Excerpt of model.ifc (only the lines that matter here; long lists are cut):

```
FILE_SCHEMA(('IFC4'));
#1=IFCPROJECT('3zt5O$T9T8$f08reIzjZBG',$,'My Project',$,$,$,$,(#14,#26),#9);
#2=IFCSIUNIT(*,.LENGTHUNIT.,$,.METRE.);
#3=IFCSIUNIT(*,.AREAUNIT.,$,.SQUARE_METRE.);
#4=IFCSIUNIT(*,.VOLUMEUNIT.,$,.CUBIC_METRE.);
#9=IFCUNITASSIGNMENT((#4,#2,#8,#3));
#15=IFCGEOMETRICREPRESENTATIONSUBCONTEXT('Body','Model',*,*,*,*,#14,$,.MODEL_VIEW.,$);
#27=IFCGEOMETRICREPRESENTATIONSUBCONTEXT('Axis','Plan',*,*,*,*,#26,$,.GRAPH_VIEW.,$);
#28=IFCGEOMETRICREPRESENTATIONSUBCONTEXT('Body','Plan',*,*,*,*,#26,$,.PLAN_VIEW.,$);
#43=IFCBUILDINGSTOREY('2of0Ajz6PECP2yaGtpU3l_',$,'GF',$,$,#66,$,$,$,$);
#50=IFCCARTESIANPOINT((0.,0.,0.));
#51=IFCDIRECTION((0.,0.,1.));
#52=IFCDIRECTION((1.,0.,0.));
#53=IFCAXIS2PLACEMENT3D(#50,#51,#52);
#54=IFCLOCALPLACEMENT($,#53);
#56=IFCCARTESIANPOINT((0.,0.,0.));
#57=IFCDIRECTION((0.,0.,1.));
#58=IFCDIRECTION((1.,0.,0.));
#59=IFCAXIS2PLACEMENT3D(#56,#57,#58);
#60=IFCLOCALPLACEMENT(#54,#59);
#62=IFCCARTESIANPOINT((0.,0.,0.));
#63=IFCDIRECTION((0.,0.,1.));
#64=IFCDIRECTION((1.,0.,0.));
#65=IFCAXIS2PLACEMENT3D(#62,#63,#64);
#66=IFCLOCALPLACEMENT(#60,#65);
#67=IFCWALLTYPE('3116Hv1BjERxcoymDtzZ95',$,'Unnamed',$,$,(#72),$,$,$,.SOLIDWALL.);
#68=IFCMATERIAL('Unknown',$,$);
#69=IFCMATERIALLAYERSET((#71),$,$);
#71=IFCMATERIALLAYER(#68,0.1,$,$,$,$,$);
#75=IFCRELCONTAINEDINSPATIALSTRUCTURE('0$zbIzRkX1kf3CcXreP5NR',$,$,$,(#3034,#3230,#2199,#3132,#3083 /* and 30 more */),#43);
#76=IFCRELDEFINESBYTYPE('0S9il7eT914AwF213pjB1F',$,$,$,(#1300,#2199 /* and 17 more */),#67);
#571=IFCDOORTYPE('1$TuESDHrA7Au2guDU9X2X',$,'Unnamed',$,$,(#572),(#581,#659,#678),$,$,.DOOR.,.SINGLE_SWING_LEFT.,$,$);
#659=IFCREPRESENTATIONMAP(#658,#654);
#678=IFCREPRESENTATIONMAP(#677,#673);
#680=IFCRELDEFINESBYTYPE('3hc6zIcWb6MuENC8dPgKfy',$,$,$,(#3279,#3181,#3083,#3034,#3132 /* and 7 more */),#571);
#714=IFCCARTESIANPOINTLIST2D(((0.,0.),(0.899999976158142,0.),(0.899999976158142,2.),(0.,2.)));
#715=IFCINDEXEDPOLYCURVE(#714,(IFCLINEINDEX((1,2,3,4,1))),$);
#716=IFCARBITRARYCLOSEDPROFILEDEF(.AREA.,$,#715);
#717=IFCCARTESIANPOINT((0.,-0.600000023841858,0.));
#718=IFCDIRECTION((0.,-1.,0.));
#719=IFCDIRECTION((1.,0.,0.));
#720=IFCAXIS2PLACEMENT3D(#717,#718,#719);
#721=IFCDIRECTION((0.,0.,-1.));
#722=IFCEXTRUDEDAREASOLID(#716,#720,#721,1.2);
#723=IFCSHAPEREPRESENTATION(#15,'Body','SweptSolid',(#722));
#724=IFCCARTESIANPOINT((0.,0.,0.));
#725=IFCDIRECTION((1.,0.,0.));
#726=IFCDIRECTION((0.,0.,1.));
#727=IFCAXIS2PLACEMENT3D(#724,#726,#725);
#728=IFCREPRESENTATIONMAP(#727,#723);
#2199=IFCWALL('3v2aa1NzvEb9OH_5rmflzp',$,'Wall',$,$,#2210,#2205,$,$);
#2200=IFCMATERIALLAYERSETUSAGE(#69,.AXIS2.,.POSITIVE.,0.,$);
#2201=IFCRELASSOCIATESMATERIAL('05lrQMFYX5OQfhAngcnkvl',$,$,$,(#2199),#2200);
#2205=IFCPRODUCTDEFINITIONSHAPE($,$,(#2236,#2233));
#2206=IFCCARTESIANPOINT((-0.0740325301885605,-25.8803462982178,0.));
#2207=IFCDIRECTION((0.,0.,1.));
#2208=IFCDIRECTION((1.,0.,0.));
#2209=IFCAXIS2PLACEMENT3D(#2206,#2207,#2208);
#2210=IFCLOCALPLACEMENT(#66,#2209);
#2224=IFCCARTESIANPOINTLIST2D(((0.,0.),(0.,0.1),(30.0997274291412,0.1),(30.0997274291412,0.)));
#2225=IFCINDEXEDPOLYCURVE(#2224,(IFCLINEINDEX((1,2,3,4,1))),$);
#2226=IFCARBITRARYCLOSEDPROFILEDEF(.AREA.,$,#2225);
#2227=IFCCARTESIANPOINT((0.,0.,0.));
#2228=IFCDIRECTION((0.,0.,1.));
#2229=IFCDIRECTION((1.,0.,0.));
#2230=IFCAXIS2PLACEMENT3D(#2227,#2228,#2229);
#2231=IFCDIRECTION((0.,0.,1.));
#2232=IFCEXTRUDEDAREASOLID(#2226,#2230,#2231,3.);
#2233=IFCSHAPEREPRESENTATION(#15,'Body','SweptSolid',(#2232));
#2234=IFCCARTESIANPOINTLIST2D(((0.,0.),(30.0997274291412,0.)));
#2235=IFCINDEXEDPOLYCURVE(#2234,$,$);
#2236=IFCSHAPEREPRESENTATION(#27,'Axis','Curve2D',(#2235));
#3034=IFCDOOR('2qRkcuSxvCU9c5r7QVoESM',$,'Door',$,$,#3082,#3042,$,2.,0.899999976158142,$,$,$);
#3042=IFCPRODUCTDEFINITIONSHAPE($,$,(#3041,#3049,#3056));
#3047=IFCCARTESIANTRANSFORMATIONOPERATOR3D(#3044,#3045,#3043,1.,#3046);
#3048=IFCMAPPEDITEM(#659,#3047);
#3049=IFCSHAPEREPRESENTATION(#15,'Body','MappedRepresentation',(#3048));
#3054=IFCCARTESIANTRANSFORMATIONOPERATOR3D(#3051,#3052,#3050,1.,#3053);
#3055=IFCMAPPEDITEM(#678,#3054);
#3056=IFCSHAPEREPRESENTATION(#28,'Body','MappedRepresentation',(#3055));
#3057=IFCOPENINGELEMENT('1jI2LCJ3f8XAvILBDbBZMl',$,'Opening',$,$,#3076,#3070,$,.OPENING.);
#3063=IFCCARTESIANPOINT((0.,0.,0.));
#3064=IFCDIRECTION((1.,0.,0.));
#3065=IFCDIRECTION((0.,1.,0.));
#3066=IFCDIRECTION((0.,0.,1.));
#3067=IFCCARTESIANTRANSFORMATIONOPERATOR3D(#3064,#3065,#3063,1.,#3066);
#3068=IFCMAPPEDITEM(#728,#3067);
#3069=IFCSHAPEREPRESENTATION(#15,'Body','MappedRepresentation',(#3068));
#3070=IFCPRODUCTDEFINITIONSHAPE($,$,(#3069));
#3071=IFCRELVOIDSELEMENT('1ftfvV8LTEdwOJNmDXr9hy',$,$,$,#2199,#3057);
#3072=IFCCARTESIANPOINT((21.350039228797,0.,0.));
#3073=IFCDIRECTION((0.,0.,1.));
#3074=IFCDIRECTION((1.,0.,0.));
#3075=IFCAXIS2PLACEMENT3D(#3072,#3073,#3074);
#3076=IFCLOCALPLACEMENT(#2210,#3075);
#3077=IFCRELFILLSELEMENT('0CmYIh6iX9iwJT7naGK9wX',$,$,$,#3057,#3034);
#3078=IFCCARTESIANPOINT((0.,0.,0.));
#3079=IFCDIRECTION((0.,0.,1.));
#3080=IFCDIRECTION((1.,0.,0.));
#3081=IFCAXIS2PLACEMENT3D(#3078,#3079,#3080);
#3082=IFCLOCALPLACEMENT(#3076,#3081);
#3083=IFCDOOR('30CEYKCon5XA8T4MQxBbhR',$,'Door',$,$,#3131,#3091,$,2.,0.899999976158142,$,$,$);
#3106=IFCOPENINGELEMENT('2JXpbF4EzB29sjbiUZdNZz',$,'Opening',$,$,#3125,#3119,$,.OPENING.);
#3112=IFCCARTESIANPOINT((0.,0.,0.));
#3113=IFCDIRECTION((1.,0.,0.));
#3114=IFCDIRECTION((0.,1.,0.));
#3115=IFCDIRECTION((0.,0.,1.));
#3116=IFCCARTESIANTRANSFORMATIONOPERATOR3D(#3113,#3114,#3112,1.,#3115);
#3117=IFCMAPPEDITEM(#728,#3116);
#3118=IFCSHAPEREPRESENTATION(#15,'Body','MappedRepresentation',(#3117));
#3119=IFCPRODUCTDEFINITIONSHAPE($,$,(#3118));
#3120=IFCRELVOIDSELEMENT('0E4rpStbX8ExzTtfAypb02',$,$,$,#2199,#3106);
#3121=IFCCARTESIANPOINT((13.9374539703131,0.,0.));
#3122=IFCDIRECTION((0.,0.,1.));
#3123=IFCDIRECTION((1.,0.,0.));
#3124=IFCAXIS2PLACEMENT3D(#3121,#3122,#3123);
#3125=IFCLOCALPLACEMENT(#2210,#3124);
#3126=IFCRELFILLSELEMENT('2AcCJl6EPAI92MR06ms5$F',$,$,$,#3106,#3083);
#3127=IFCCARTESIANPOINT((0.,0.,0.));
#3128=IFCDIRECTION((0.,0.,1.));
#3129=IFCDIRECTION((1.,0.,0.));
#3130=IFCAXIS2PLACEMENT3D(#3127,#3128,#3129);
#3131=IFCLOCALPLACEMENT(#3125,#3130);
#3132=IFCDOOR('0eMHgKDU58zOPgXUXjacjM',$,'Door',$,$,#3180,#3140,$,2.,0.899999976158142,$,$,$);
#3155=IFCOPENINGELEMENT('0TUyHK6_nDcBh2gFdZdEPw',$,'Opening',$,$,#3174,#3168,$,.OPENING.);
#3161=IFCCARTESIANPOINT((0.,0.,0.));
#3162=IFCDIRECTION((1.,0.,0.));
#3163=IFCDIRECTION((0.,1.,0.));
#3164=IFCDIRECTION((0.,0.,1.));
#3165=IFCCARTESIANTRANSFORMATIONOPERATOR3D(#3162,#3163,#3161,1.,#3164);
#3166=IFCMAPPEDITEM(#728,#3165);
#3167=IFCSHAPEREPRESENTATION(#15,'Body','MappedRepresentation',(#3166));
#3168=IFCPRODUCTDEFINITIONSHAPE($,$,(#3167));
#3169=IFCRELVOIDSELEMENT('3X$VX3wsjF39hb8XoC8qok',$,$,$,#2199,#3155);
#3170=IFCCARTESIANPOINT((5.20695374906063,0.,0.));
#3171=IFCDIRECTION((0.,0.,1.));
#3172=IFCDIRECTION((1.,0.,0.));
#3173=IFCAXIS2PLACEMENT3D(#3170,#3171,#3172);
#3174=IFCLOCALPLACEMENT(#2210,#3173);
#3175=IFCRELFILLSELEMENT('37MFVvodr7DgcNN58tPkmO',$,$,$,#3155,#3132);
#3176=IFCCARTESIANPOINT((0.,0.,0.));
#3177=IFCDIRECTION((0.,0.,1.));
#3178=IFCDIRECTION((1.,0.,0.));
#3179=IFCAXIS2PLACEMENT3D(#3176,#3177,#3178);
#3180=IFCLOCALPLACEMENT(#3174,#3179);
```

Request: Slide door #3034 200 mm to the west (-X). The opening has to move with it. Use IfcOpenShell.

```python
import ifcopenshell
import ifcopenshell.api.geometry
import ifcopenshell.util.placement
import ifcopenshell.util.unit

model = ifcopenshell.open("model.ifc")
unit_scale = ifcopenshell.util.unit.calculate_unit_scale(model)

door = model.by_id(3034)
opening = door.FillsVoids[0].RelatingOpeningElement
wall = opening.VoidsElements[0].RelatingBuildingElement

wall_matrix = ifcopenshell.util.placement.get_local_placement(wall.ObjectPlacement)
shift = wall_matrix[:3, 0] * -0.2 / unit_scale
before = ifcopenshell.util.placement.get_local_placement(door.ObjectPlacement)[:3, 3].copy()

# The door is placed relative to its opening, so it follows when the opening moves.
matrix = ifcopenshell.util.placement.get_local_placement(opening.ObjectPlacement)
matrix[:3, 3] += shift
ifcopenshell.api.geometry.edit_object_placement(
    model, product=opening, matrix=matrix, is_si=False, should_transform_children=True
)

after = ifcopenshell.util.placement.get_local_placement(door.ObjectPlacement)[:3, 3]
print("door moved by", (after - before).round(3) + 0.0)

model.write("model_edited.ifc")
```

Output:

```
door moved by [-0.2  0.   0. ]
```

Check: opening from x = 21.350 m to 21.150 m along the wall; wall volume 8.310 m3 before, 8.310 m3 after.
